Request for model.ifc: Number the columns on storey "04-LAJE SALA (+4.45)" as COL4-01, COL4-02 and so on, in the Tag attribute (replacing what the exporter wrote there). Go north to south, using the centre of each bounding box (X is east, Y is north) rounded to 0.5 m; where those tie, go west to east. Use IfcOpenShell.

First a look at what the model holds.

```python
import ifcopenshell
import ifcopenshell.util.element
import ifcopenshell.util.placement

model = ifcopenshell.open("model.ifc")
print(model.schema)
storey = next(s for s in model.by_type("IfcBuildingStorey") if s.Name == "04-LAJE SALA (+4.45)")
columns = [e for e in ifcopenshell.util.element.get_decomposition(storey) if e.is_a("IfcColumn")]
for e in sorted(columns, key=lambda e: e.id()):
    origin = ifcopenshell.util.placement.get_local_placement(e.ObjectPlacement)[:3, 3]
    print(e.id(), e.Tag, e.Name, origin.round(2) + 0.0, sep=" | ")
```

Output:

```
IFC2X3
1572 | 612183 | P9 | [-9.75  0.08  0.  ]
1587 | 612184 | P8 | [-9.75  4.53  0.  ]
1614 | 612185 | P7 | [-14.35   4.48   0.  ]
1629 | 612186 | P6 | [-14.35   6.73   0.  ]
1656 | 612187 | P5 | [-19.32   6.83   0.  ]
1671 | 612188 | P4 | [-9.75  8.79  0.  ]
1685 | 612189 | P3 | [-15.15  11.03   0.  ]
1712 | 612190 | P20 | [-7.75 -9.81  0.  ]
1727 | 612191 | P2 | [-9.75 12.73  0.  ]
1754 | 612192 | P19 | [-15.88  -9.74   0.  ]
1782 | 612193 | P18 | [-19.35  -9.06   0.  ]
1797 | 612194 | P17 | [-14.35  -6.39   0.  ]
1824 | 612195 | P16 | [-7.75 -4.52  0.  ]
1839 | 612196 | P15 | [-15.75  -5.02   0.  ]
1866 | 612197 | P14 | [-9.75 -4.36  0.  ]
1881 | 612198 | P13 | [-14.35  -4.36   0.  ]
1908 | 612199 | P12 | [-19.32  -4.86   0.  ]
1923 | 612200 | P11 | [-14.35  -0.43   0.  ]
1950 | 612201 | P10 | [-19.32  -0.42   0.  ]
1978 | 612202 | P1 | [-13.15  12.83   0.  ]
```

```python
import ifcopenshell
import ifcopenshell.geom
import ifcopenshell.util.element
import ifcopenshell.util.shape

model = ifcopenshell.open("model.ifc")
settings = ifcopenshell.geom.settings()
settings.set("use-world-coords", True)


def centre(element):
    shape = ifcopenshell.geom.create_shape(settings, element)
    return ifcopenshell.util.shape.get_bbox_centroid(shape.geometry)


storey = next(s for s in model.by_type("IfcBuildingStorey") if s.Name == "04-LAJE SALA (+4.45)")
columns = [e for e in ifcopenshell.util.element.get_decomposition(storey) if e.is_a("IfcColumn")]

# Insertion points can sit at a corner or the storey origin, so sort by the geometry (in metres).
centres = {e: centre(e) for e in columns}
columns.sort(key=lambda e: (-round(centres[e][1] / 0.5), centres[e][0]))

for i, e in enumerate(columns, start=1):
    number = f"COL4-{i:02d}"
    e.Tag = number
    print(e.id(), number)

model.write("model_v2.ifc")
```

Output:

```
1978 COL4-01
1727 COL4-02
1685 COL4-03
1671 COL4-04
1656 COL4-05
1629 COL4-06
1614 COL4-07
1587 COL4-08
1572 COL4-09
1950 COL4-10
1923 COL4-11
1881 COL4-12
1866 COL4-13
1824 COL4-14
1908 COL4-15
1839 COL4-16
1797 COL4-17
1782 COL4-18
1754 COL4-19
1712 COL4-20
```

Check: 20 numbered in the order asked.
